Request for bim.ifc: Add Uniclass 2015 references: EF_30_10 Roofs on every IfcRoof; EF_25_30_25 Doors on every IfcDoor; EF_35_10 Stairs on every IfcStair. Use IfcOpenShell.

First a look at what the model holds.

```python
import ifcopenshell

model = ifcopenshell.open("bim.ifc")
print(model.schema)
print("classifications:", [c.Name for c in model.by_type("IfcClassification")])
for ifc_class in ("IfcDoor", "IfcRoof", "IfcStair", "IfcWall", "IfcWindow"):
    print(ifc_class, len(model.by_type(ifc_class)))
```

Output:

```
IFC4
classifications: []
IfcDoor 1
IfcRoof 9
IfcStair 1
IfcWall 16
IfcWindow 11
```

```python
import ifcopenshell
import ifcopenshell.api.classification

model = ifcopenshell.open("bim.ifc")

system = ifcopenshell.api.classification.add_classification(model, classification="Uniclass 2015")

codes = {
    "IfcRoof": ("EF_30_10", "Roofs"),
    "IfcDoor": ("EF_25_30_25", "Doors"),
    "IfcStair": ("EF_35_10", "Stairs"),
}
for ifc_class, (code, name) in codes.items():
    products = model.by_type(ifc_class)
    ifcopenshell.api.classification.add_reference(
        model, products=products, classification=system, identification=code, name=name
    )
    print(code, len(products))

model.write("bim_rev.ifc")
```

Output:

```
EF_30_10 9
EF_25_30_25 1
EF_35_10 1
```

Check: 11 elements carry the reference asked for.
